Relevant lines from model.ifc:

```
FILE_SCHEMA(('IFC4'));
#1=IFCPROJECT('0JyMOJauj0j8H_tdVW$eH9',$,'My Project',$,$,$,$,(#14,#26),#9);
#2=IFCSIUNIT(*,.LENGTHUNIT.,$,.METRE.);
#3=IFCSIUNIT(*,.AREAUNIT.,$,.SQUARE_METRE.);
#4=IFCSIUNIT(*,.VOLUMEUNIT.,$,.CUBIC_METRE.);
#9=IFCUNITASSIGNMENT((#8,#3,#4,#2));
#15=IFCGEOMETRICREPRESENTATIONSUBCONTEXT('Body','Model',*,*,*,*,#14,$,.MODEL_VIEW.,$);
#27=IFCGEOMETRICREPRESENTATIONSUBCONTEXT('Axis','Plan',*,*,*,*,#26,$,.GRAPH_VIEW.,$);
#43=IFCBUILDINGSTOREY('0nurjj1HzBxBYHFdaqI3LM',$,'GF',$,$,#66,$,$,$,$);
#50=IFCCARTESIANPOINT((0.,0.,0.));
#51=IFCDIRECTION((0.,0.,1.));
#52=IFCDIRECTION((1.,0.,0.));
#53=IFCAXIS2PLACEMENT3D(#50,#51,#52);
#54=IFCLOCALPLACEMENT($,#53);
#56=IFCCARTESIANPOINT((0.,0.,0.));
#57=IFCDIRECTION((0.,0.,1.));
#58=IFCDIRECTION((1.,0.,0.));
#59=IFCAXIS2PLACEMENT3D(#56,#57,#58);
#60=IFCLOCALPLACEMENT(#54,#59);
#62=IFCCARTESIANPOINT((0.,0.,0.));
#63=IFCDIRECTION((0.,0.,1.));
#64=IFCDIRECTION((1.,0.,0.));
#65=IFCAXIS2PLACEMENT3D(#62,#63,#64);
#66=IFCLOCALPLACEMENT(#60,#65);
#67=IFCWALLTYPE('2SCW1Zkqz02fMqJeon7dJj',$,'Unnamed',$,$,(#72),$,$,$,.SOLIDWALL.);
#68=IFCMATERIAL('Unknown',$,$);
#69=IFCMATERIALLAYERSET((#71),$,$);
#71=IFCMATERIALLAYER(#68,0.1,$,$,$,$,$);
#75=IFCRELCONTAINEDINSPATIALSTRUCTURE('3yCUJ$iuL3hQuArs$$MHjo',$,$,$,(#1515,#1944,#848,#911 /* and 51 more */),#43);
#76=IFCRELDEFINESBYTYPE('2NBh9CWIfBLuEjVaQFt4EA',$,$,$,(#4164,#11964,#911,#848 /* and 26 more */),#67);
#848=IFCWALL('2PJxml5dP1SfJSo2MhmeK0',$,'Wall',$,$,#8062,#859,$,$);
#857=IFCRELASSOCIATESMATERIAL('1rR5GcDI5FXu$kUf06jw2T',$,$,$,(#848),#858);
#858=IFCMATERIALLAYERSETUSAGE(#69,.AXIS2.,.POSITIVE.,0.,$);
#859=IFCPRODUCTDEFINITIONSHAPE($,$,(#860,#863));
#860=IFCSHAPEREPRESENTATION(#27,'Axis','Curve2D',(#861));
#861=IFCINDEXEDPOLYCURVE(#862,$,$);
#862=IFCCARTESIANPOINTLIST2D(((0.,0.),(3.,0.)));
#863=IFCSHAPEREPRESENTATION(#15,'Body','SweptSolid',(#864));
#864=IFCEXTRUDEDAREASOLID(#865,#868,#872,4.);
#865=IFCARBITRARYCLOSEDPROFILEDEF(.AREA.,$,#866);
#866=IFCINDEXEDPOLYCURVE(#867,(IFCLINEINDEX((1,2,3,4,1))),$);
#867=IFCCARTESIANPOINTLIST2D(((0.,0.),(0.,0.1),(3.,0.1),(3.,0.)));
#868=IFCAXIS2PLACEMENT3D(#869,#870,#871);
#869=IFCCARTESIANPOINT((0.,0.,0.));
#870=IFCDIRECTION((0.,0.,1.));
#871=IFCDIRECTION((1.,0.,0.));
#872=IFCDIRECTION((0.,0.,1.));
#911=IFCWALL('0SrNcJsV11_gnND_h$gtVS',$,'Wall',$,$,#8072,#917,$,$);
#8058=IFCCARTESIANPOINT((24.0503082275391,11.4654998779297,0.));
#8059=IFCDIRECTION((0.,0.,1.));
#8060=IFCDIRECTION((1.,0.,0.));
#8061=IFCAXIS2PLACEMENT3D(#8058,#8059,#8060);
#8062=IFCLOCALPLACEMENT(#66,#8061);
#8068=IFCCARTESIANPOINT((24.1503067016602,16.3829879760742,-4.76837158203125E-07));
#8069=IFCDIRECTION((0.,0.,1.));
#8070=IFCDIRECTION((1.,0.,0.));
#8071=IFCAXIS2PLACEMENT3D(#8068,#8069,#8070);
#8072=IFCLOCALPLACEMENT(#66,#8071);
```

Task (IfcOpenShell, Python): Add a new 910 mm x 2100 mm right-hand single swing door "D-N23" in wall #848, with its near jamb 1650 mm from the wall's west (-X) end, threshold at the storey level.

```python
import numpy as np
import ifcopenshell
import ifcopenshell.api.feature
import ifcopenshell.api.geometry
import ifcopenshell.api.root
import ifcopenshell.api.spatial
import ifcopenshell.geom
import ifcopenshell.util.element
import ifcopenshell.util.placement
import ifcopenshell.util.representation
import ifcopenshell.util.shape
import ifcopenshell.util.unit

model = ifcopenshell.open("model.ifc")
unit_scale = ifcopenshell.util.unit.calculate_unit_scale(model)
settings = ifcopenshell.geom.settings()


def volume(element):
    """Net volume in cubic metres, openings subtracted."""
    shape = ifcopenshell.geom.create_shape(settings, element)
    return ifcopenshell.util.shape.get_volume(shape.geometry)


wall = model.by_guid("2PJxml5dP1SfJSo2MhmeK0")
storey = ifcopenshell.util.element.get_container(wall, ifc_class="IfcBuildingStorey")
context = ifcopenshell.util.representation.get_context(model, "Model", "Body", "MODEL_VIEW")
before = volume(wall)

width, height, from_end, sill = 0.91, 2.1, 1.65, 0.0  # metres

# The wall runs along its own X axis, and the end named is its -X end.
wall_shape = ifcopenshell.geom.create_shape(settings, wall)
x, y, z = ifcopenshell.util.shape.get_vertices(wall_shape.geometry).T
start = x.min() + from_end
face, thickness = float(y.min()), float(y.max() - y.min())
wall_matrix = ifcopenshell.util.placement.get_local_placement(wall.ObjectPlacement)
level = ifcopenshell.util.placement.get_local_placement(storey.ObjectPlacement)[2, 3]


def in_wall(x, y):
    """Placement at x, y metres in the wall's axes, at sill height."""
    matrix = wall_matrix.copy()
    matrix[:, 3] = wall_matrix @ np.array([x / unit_scale, y / unit_scale, 0.0, 1.0])
    matrix[2, 3] = level + sill / unit_scale
    return matrix


# Opening: a box that overshoots both wall faces by 50 mm.
opening = ifcopenshell.api.root.create_entity(model, ifc_class="IfcOpeningElement", predefined_type="OPENING")
box = ifcopenshell.api.geometry.add_wall_representation(
    model, context=context, length=width, height=height, thickness=thickness + 0.1
)
ifcopenshell.api.geometry.assign_representation(model, product=opening, representation=box)
ifcopenshell.api.geometry.edit_object_placement(model, product=opening, matrix=in_wall(start, face - 0.05), is_si=False)
ifcopenshell.api.feature.add_feature(model, feature=opening, element=wall)

door = ifcopenshell.api.root.create_entity(model, ifc_class="IfcDoor", name="D-N23", predefined_type="DOOR")
door.OverallWidth, door.OverallHeight = width / unit_scale, height / unit_scale
door.OperationType = "SINGLE_SWING_RIGHT"
body = ifcopenshell.api.geometry.add_door_representation(
    model,
    context=context,
    overall_width=door.OverallWidth,
    overall_height=door.OverallHeight,
    operation_type="SINGLE_SWING_RIGHT",
    lining_properties={"LiningDepth": thickness / unit_scale, "ThresholdDepth": thickness / unit_scale},
)
ifcopenshell.api.geometry.assign_representation(model, product=door, representation=body)
ifcopenshell.api.spatial.assign_container(model, products=[door], relating_structure=storey)
ifcopenshell.api.feature.add_filling(model, opening=opening, element=door)

# The lining spans the wall, so the door starts at the wall face.
ifcopenshell.api.geometry.edit_object_placement(model, product=door, matrix=in_wall(start, face), is_si=False)

after = volume(wall)

print(f"wall volume {before:.3f} -> {after:.3f} m3")

model.write("model-out.ifc")
```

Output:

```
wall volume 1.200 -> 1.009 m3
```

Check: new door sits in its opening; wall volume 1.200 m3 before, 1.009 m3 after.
